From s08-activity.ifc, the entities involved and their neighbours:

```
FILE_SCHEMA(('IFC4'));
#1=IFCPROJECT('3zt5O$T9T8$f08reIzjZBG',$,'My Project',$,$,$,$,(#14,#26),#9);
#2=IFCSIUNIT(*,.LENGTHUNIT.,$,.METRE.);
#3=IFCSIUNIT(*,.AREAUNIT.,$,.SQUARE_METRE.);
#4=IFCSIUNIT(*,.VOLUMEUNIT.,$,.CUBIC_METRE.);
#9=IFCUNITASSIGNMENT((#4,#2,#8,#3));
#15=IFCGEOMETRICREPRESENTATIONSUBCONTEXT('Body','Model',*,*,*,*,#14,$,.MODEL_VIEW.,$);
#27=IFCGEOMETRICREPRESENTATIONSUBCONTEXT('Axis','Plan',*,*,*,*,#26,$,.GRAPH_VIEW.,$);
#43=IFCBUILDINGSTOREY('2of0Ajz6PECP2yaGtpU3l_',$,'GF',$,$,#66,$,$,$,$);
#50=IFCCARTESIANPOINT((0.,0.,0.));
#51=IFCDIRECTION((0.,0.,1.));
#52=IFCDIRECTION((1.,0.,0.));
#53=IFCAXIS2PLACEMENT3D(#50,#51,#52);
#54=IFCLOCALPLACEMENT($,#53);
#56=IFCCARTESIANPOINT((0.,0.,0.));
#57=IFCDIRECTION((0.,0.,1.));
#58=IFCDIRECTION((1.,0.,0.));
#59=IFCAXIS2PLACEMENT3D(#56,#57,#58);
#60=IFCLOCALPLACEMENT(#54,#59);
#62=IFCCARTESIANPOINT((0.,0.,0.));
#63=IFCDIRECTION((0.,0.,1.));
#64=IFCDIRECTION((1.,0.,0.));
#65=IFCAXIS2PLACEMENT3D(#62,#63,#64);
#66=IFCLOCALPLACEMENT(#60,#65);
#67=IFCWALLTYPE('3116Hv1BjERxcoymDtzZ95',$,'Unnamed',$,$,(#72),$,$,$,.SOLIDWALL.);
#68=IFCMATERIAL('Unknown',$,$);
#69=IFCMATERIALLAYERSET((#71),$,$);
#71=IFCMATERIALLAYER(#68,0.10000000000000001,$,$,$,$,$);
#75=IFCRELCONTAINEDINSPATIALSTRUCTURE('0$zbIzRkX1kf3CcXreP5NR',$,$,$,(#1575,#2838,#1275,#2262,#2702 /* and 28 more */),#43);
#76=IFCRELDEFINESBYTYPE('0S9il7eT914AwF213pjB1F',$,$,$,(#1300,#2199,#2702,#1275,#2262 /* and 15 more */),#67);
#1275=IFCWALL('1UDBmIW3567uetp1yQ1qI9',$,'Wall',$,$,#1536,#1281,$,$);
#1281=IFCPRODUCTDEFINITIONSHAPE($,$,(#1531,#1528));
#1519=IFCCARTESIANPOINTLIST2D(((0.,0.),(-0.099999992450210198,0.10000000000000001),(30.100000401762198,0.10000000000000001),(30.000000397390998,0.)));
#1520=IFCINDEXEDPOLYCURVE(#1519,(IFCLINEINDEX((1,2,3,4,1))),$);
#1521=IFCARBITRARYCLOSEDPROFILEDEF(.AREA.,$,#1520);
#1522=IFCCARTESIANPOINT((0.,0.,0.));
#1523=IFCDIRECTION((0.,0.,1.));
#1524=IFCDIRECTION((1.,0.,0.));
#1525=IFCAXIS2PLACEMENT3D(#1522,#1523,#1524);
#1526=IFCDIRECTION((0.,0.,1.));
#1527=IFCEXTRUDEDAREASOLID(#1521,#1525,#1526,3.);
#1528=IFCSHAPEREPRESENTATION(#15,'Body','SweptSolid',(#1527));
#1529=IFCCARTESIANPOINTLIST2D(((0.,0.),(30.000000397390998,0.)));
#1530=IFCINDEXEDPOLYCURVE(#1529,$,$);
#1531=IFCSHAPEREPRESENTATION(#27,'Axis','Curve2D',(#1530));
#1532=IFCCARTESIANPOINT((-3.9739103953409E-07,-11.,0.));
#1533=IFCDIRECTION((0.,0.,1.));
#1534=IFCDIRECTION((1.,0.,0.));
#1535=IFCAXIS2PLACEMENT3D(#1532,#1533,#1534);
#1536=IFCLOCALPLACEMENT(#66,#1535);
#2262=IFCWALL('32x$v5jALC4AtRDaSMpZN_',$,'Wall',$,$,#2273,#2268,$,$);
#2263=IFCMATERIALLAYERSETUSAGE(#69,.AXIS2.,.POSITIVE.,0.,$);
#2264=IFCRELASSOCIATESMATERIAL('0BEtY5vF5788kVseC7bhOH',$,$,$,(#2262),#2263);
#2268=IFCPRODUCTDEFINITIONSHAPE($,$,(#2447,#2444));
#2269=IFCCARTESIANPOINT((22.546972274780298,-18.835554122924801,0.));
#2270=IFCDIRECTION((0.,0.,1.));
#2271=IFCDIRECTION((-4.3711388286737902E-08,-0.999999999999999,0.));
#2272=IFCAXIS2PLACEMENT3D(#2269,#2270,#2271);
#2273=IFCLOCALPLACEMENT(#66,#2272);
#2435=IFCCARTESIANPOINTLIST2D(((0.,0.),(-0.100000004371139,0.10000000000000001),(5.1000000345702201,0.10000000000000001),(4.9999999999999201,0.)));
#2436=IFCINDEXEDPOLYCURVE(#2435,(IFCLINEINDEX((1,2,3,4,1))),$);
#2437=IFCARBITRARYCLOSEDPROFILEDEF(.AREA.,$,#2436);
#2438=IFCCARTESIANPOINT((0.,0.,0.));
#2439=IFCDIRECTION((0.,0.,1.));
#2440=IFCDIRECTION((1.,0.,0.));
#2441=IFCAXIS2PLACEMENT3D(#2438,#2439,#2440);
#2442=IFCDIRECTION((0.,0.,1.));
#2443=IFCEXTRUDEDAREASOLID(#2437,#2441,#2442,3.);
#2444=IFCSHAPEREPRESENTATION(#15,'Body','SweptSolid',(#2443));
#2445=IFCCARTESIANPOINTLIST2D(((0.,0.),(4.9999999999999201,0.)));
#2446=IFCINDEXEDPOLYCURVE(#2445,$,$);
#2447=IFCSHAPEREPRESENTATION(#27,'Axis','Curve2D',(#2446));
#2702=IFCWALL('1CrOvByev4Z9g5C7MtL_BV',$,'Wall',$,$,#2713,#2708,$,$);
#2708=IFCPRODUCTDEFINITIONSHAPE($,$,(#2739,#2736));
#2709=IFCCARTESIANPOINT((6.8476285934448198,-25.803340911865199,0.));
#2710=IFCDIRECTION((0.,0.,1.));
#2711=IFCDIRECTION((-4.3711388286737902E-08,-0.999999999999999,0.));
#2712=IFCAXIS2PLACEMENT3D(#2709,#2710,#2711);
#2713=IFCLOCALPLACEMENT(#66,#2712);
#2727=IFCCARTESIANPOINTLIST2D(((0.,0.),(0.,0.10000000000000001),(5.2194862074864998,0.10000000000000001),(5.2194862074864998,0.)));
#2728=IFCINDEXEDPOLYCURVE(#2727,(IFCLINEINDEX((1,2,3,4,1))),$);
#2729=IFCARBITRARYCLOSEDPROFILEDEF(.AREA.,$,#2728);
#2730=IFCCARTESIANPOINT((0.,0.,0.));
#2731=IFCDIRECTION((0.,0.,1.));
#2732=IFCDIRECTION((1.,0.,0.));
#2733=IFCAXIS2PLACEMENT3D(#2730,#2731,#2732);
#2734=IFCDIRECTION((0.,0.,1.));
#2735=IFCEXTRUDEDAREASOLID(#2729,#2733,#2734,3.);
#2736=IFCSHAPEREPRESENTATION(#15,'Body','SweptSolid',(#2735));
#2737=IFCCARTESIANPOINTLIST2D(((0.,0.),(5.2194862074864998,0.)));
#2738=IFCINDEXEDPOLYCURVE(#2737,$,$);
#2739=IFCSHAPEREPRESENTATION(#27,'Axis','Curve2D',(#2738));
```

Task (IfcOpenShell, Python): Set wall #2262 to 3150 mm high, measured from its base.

```python
import ifcopenshell
import ifcopenshell.geom
import ifcopenshell.util.representation
import ifcopenshell.util.shape
import ifcopenshell.util.unit

model = ifcopenshell.open("s08-activity.ifc")
unit_scale = ifcopenshell.util.unit.calculate_unit_scale(model)
settings = ifcopenshell.geom.settings()


def volume(element):
    """Net volume in cubic metres, openings subtracted."""
    shape = ifcopenshell.geom.create_shape(settings, element)
    return ifcopenshell.util.shape.get_volume(shape.geometry)


wall = model.by_guid("32x$v5jALC4AtRDaSMpZN_")
before = volume(wall)

body = ifcopenshell.util.representation.get_representation(wall, "Model", "Body")
solid = body.Items[0]
old_height = solid.Depth
solid.Depth = 3.15 / unit_scale
after = volume(wall)

print(f"height {old_height:g} -> {solid.Depth:g}, volume {before:.3f} -> {after:.3f} m3")

model.write("s08-activity_v2.ifc")
```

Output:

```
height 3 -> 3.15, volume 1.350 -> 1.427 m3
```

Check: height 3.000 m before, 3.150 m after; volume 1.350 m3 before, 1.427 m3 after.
